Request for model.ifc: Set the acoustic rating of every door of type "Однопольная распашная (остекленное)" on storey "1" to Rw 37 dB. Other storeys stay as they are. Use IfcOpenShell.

First a look at what the model holds.

```python
import ifcopenshell
import ifcopenshell.util.element

model = ifcopenshell.open("model.ifc")
print(model.schema)
storey = next(s for s in model.by_type("IfcBuildingStorey") if s.Name == "1")
doors = [e for e in ifcopenshell.util.element.get_decomposition(storey) if e.is_a("IfcDoor")]
seen = {}
for e in doors:
    element_type = ifcopenshell.util.element.get_type(e)
    key = (element_type.Name if element_type != e and element_type else None, ifcopenshell.util.element.get_pset(e, "Pset_DoorCommon", "AcousticRating"))
    seen[key] = seen.get(key, 0) + 1
for (name, value), count in sorted(seen.items(), key=str):
    print(count, "x", name, "|", value)
```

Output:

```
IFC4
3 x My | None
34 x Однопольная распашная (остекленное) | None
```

```python
import ifcopenshell
import ifcopenshell.api.pset
import ifcopenshell.util.element

model = ifcopenshell.open("model.ifc")

storey = next(s for s in model.by_type("IfcBuildingStorey") if s.Name == "1")
doors = [e for e in ifcopenshell.util.element.get_decomposition(storey) if e.is_a("IfcDoor")]

count = 0
for e in doors:
    element_type = ifcopenshell.util.element.get_type(e)
    if element_type in (None, e) or element_type.Name != "Однопольная распашная (остекленное)":
        continue
    # add_pset returns the element's existing set when there is one.
    pset = ifcopenshell.api.pset.add_pset(model, product=e, name="Pset_DoorCommon")
    ifcopenshell.api.pset.edit_pset(model, pset=pset, properties={"AcousticRating": "Rw 37 dB"})
    count += 1

print(count, "doors updated")

model.write("model-out.ifc")
```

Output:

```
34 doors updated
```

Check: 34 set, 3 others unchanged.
